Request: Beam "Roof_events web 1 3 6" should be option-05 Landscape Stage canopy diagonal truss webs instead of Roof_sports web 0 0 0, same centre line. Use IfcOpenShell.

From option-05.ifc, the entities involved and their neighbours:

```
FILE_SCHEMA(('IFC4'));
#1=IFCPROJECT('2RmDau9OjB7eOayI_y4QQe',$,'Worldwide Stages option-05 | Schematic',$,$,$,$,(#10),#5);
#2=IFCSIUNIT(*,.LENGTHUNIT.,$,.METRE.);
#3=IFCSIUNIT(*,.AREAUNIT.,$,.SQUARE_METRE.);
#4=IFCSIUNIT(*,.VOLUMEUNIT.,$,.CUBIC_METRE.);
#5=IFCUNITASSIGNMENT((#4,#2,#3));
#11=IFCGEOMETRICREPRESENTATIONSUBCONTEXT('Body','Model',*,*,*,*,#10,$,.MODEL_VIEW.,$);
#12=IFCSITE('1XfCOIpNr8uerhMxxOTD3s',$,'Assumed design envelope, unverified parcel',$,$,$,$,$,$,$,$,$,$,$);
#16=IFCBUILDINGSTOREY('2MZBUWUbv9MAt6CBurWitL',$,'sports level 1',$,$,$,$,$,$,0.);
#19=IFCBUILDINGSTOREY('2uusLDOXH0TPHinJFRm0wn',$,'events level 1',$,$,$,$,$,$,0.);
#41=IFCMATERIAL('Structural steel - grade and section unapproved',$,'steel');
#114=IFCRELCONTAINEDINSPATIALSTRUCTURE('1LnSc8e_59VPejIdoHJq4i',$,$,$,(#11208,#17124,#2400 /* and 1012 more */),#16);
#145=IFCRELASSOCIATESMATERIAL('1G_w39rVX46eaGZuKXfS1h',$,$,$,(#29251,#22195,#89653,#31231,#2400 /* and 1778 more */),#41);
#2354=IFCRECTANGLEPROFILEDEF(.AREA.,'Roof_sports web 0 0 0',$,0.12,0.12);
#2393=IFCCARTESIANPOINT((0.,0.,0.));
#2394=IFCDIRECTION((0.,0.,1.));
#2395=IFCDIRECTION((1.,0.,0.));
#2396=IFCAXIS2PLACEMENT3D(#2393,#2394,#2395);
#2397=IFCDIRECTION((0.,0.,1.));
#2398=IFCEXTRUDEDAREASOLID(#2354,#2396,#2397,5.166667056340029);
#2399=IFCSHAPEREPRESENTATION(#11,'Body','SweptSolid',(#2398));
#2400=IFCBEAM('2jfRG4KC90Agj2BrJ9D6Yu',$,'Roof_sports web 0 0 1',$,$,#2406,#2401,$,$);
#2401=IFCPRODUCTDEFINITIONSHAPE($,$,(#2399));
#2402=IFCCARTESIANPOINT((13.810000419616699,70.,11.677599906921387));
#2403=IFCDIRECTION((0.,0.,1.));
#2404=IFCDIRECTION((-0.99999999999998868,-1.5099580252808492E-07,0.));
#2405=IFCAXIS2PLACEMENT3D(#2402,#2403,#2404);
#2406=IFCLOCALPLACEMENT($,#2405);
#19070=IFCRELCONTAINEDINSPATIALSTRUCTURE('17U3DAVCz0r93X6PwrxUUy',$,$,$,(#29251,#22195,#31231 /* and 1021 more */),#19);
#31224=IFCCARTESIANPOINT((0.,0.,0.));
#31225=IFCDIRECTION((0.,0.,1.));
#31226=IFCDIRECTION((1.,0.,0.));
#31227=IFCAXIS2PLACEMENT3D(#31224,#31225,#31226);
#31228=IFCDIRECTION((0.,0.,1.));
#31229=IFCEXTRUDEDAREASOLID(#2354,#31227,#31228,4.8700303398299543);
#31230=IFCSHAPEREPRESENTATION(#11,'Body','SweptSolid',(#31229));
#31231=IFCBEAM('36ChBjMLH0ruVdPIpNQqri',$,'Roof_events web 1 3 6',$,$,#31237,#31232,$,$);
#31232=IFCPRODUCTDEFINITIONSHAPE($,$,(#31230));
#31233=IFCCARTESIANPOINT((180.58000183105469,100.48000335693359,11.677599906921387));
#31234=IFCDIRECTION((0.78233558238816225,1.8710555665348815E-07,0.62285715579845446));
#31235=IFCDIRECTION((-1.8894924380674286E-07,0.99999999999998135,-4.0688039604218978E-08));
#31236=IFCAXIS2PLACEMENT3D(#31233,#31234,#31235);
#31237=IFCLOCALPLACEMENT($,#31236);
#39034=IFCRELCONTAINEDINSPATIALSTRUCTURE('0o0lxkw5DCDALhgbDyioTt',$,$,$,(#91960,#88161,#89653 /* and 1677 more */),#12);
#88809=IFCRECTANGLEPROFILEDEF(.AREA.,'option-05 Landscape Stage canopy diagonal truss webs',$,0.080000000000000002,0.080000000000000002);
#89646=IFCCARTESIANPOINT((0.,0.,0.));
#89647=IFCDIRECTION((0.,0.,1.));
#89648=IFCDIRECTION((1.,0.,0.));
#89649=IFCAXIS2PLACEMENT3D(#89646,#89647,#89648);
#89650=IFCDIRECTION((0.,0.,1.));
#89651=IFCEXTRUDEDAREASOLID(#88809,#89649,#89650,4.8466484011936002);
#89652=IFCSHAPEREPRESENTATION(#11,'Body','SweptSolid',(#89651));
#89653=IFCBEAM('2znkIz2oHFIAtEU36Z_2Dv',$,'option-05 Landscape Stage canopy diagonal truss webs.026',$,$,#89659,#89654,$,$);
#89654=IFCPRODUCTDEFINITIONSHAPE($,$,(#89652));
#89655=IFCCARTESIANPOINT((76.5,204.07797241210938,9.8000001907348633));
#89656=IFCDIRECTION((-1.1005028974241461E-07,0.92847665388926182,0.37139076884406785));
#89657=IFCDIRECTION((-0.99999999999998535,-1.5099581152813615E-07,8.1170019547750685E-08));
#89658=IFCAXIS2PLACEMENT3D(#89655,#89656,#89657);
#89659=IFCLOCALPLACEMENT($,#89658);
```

```python
import ifcopenshell
import ifcopenshell.util.element
import ifcopenshell.util.representation

model = ifcopenshell.open("option-05.ifc")

member = model.by_guid("36ChBjMLH0ruVdPIpNQqri")
source = next(p for p in model.by_type("IfcRectangleProfileDef") if p.ProfileName == "option-05 Landscape Stage canopy diagonal truss webs")

body = ifcopenshell.util.representation.get_representation(member, "Model", "Body")
solid = body.Items[0]
old_profile = solid.SweptArea

# Copy the section's sizes but keep this member's own profile position.
profile = ifcopenshell.util.element.copy(model, source)
profile.Position = old_profile.Position
solid.SweptArea = profile
if not model.get_total_inverses(old_profile):
    ifcopenshell.util.element.remove_deep2(model, old_profile)

print(solid.SweptArea)

model.write("option-05_rev.ifc")
```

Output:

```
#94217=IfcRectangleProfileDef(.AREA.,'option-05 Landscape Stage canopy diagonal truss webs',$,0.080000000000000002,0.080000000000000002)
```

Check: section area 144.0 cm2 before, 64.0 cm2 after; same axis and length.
